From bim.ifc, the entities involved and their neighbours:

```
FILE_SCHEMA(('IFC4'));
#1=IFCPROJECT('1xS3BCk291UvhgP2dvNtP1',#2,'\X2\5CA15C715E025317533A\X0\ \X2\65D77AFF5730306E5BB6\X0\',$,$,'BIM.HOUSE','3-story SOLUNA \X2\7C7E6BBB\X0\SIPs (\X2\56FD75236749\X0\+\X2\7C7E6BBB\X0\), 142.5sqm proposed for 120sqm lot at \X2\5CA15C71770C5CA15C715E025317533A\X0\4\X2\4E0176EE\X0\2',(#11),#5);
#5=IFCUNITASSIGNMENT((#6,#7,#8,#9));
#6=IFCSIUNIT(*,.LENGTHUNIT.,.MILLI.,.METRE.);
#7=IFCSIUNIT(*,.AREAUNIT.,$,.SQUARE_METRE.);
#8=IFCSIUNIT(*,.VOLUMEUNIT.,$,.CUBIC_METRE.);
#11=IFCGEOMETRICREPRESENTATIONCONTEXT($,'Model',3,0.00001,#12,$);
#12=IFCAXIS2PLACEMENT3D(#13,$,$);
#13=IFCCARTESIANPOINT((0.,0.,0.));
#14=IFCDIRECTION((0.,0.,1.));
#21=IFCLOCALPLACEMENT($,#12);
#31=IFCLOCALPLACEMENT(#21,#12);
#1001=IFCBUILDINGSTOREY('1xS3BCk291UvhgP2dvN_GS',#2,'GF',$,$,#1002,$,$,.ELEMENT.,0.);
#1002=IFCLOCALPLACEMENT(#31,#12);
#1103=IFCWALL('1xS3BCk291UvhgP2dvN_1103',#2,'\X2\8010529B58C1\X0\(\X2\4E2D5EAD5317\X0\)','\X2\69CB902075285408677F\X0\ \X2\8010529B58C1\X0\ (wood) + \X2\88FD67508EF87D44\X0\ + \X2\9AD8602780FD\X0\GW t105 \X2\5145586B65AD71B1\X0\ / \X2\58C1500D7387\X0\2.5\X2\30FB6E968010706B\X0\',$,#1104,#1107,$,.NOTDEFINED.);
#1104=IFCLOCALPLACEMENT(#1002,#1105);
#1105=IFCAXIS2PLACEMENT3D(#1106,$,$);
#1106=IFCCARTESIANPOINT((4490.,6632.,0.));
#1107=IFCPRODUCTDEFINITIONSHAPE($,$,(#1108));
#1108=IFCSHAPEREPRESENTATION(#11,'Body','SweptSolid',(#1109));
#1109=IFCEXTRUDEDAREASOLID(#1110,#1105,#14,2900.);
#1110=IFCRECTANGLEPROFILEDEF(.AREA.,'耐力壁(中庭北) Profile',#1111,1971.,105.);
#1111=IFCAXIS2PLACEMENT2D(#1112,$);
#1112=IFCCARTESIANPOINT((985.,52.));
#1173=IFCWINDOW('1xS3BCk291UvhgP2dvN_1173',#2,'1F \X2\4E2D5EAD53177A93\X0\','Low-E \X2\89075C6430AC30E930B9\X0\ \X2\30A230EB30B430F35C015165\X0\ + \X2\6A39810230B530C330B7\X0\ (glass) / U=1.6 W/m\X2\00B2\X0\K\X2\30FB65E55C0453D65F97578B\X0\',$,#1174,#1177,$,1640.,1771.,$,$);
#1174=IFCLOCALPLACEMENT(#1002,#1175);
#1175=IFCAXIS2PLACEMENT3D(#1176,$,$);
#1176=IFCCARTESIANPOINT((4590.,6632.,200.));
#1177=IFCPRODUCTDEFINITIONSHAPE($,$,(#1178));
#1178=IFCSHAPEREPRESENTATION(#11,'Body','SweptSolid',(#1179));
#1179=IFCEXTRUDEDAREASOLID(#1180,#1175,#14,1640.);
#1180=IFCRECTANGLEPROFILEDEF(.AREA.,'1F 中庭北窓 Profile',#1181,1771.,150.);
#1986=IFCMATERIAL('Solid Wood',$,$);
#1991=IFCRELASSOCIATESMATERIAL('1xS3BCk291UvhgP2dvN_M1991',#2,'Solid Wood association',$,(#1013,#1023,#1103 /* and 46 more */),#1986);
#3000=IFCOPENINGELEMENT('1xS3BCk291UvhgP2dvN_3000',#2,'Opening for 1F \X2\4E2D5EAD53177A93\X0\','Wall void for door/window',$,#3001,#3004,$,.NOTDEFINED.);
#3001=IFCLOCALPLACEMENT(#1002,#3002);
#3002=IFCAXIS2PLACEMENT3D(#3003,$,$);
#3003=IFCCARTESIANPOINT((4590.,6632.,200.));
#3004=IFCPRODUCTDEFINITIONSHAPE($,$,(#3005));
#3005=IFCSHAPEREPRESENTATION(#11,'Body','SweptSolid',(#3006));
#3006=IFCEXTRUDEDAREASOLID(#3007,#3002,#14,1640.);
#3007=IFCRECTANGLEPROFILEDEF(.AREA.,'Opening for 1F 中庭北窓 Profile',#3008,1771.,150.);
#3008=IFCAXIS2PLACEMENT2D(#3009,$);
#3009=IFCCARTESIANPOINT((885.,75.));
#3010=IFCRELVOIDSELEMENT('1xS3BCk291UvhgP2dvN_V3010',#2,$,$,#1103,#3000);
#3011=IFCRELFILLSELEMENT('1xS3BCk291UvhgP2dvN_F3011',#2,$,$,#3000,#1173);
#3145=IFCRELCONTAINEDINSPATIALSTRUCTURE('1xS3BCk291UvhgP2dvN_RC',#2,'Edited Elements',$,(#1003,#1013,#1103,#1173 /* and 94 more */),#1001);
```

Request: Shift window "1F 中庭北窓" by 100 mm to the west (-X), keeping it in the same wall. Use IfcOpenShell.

```python
import ifcopenshell
import ifcopenshell.api.geometry
import ifcopenshell.util.placement
import ifcopenshell.util.unit

model = ifcopenshell.open("bim.ifc")
unit_scale = ifcopenshell.util.unit.calculate_unit_scale(model)

window = model.by_guid("1xS3BCk291UvhgP2dvN_1173")
opening = window.FillsVoids[0].RelatingOpeningElement
wall = opening.VoidsElements[0].RelatingBuildingElement

wall_matrix = ifcopenshell.util.placement.get_local_placement(wall.ObjectPlacement)
shift = wall_matrix[:3, 0] * -0.1 / unit_scale
before = ifcopenshell.util.placement.get_local_placement(window.ObjectPlacement)[:3, 3].copy()

# The window is not placed relative to its opening, so move both.
for product in (opening, window):
    matrix = ifcopenshell.util.placement.get_local_placement(product.ObjectPlacement)
    matrix[:3, 3] += shift
    ifcopenshell.api.geometry.edit_object_placement(model, product=product, matrix=matrix, is_si=False)

after = ifcopenshell.util.placement.get_local_placement(window.ObjectPlacement)[:3, 3]
print("window moved by", (after - before).round(3) + 0.0)

model.write("bim_rev.ifc")
```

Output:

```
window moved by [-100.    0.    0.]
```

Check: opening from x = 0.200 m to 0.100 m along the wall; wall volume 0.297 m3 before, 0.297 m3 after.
